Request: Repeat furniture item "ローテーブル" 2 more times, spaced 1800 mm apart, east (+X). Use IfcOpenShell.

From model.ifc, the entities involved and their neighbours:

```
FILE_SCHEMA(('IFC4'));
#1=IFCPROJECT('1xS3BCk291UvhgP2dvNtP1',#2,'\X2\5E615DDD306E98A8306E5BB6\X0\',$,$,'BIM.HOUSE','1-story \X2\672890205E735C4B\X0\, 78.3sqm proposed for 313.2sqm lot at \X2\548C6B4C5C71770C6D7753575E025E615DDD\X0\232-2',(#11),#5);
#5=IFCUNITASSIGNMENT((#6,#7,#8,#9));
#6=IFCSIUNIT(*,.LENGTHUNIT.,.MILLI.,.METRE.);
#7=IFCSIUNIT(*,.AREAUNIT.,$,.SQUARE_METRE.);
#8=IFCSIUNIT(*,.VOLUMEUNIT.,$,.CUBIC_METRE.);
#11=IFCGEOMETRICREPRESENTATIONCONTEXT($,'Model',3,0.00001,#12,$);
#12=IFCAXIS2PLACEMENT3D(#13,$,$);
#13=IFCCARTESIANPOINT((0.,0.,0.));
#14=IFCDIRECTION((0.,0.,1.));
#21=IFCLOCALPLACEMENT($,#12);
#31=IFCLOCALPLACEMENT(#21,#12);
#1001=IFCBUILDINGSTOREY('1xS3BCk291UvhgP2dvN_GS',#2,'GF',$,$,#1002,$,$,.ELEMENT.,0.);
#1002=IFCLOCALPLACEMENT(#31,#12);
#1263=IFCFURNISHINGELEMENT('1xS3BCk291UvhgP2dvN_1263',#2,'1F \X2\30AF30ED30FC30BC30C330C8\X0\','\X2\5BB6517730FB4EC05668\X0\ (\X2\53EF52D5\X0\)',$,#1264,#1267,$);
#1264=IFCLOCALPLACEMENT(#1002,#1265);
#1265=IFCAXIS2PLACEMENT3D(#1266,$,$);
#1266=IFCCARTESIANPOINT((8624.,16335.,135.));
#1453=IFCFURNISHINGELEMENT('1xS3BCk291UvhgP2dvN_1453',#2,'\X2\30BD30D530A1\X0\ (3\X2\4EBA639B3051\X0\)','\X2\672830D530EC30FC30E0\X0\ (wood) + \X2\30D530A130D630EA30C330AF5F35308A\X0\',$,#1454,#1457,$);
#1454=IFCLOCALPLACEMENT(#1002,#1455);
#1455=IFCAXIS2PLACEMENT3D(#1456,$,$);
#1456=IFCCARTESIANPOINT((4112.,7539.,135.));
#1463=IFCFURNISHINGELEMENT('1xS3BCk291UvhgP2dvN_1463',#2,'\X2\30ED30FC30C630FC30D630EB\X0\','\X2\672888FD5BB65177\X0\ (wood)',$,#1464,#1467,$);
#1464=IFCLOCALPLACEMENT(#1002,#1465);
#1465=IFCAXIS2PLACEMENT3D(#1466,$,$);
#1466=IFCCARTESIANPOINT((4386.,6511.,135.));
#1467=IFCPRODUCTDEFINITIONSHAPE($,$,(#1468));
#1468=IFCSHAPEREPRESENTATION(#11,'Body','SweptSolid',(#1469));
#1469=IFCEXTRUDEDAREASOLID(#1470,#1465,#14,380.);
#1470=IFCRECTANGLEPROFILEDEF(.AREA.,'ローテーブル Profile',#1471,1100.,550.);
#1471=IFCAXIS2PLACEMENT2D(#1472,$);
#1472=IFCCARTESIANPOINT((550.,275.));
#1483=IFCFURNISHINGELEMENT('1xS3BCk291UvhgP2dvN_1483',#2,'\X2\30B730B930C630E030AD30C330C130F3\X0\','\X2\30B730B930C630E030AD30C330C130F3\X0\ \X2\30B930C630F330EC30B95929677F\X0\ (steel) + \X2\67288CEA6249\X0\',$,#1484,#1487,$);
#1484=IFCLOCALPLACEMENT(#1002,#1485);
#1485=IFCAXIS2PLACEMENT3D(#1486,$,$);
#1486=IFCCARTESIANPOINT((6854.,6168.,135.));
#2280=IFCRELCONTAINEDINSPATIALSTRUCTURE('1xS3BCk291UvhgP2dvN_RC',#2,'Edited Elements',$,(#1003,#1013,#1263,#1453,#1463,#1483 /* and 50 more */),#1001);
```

```python
import numpy as np
import ifcopenshell
import ifcopenshell.api.geometry
import ifcopenshell.api.root
import ifcopenshell.util.element
import ifcopenshell.util.placement

model = ifcopenshell.open("model.ifc")


def reuse_history(source, copy):
    """copy_class also copies each property set's owner history, people and application; keep the originals."""
    for rel in copy.IsDefinedBy:
        if rel.is_a("IfcRelDefinesByProperties") and (history := rel.RelatingPropertyDefinition.OwnerHistory):
            rel.RelatingPropertyDefinition.OwnerHistory = source.OwnerHistory
            ifcopenshell.util.element.remove_deep2(model, history)


source = model.by_id(1463)
base = ifcopenshell.util.placement.get_local_placement(source.ObjectPlacement)
step = np.array([1.0, 0.0, 0.0]) * 1800.0

for i in range(1, 3):
    copy = ifcopenshell.api.root.copy_class(model, product=source)
    copy.Representation = ifcopenshell.util.element.copy_deep(
        model, source.Representation, exclude=["IfcGeometricRepresentationContext", "IfcRepresentationMap"]
    )
    reuse_history(source, copy)
    matrix = base.copy()
    matrix[:3, 3] += i * step
    print("added at", matrix[:3, 3].round(3) + 0.0)
    ifcopenshell.api.geometry.edit_object_placement(model, product=copy, matrix=matrix, is_si=False)

model.write("model_rev.ifc")
```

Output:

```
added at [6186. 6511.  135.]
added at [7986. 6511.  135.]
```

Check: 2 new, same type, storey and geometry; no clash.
